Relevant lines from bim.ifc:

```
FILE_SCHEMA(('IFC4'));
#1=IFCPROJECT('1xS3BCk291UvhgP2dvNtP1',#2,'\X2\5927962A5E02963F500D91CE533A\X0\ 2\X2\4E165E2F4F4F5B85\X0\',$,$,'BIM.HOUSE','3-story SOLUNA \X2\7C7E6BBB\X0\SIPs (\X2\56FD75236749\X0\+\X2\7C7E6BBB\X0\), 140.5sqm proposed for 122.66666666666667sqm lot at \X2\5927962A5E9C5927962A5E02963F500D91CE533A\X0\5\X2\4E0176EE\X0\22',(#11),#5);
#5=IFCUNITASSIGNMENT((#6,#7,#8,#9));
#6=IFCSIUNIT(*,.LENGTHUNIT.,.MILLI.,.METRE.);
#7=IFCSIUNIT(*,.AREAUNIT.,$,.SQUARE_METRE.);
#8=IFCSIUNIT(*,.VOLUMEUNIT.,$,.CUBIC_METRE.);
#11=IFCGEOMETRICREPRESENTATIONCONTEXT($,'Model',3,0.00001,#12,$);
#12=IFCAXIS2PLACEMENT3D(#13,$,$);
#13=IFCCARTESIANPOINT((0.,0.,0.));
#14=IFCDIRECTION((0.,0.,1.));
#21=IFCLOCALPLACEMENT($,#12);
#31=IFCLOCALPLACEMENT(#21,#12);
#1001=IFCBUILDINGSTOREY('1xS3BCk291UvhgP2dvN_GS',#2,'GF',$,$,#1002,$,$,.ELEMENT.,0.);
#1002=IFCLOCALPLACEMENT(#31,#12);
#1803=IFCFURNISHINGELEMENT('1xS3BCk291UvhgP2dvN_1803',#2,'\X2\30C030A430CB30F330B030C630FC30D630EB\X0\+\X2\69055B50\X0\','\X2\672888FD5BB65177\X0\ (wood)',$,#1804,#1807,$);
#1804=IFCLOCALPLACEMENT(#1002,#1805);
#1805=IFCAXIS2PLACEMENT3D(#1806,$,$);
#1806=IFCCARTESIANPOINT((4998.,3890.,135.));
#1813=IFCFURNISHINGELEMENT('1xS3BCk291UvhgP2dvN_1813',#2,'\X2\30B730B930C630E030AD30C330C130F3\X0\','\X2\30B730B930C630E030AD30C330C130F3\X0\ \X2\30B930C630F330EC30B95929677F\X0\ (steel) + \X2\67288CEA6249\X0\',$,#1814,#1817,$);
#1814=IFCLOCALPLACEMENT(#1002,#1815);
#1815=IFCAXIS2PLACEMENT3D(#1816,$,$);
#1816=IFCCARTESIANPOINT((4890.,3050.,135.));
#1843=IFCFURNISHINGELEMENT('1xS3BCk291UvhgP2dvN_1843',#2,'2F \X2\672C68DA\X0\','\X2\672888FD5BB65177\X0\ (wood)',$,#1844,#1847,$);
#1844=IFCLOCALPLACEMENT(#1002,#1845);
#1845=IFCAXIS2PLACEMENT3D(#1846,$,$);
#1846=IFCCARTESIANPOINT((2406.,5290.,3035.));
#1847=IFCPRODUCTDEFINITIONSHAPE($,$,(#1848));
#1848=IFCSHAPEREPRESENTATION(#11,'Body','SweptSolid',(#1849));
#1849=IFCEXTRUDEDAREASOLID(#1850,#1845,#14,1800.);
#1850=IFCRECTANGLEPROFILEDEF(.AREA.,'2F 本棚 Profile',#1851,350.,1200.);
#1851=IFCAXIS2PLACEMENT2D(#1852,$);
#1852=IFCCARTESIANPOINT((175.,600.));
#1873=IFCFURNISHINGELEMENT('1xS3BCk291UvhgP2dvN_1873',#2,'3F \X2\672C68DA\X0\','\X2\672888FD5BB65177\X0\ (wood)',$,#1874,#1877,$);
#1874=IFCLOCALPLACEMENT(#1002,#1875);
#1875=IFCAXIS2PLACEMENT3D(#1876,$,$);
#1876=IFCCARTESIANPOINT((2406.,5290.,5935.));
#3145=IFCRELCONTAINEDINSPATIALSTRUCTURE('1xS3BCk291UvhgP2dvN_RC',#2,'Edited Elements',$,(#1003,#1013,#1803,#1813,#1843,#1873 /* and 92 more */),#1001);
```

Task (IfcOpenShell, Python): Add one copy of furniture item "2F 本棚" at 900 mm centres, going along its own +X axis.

```python
import ifcopenshell
import ifcopenshell.api.geometry
import ifcopenshell.api.root
import ifcopenshell.util.element
import ifcopenshell.util.placement

model = ifcopenshell.open("bim.ifc")


def reuse_history(source, copy):
    """copy_class also copies each property set's owner history, people and application; keep the originals."""
    for rel in copy.IsDefinedBy:
        if rel.is_a("IfcRelDefinesByProperties") and (history := rel.RelatingPropertyDefinition.OwnerHistory):
            rel.RelatingPropertyDefinition.OwnerHistory = source.OwnerHistory
            ifcopenshell.util.element.remove_deep2(model, history)


source = model.by_id(1843)
base = ifcopenshell.util.placement.get_local_placement(source.ObjectPlacement)
step = base[:3, 0] * 900.0

for i in range(1, 2):
    copy = ifcopenshell.api.root.copy_class(model, product=source)
    copy.Representation = ifcopenshell.util.element.copy_deep(
        model, source.Representation, exclude=["IfcGeometricRepresentationContext", "IfcRepresentationMap"]
    )
    reuse_history(source, copy)
    matrix = base.copy()
    matrix[:3, 3] += i * step
    print("added at", matrix[:3, 3].round(3) + 0.0)
    ifcopenshell.api.geometry.edit_object_placement(model, product=copy, matrix=matrix, is_si=False)

model.write("bim-out.ifc")
```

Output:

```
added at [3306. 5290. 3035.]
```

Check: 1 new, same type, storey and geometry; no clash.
